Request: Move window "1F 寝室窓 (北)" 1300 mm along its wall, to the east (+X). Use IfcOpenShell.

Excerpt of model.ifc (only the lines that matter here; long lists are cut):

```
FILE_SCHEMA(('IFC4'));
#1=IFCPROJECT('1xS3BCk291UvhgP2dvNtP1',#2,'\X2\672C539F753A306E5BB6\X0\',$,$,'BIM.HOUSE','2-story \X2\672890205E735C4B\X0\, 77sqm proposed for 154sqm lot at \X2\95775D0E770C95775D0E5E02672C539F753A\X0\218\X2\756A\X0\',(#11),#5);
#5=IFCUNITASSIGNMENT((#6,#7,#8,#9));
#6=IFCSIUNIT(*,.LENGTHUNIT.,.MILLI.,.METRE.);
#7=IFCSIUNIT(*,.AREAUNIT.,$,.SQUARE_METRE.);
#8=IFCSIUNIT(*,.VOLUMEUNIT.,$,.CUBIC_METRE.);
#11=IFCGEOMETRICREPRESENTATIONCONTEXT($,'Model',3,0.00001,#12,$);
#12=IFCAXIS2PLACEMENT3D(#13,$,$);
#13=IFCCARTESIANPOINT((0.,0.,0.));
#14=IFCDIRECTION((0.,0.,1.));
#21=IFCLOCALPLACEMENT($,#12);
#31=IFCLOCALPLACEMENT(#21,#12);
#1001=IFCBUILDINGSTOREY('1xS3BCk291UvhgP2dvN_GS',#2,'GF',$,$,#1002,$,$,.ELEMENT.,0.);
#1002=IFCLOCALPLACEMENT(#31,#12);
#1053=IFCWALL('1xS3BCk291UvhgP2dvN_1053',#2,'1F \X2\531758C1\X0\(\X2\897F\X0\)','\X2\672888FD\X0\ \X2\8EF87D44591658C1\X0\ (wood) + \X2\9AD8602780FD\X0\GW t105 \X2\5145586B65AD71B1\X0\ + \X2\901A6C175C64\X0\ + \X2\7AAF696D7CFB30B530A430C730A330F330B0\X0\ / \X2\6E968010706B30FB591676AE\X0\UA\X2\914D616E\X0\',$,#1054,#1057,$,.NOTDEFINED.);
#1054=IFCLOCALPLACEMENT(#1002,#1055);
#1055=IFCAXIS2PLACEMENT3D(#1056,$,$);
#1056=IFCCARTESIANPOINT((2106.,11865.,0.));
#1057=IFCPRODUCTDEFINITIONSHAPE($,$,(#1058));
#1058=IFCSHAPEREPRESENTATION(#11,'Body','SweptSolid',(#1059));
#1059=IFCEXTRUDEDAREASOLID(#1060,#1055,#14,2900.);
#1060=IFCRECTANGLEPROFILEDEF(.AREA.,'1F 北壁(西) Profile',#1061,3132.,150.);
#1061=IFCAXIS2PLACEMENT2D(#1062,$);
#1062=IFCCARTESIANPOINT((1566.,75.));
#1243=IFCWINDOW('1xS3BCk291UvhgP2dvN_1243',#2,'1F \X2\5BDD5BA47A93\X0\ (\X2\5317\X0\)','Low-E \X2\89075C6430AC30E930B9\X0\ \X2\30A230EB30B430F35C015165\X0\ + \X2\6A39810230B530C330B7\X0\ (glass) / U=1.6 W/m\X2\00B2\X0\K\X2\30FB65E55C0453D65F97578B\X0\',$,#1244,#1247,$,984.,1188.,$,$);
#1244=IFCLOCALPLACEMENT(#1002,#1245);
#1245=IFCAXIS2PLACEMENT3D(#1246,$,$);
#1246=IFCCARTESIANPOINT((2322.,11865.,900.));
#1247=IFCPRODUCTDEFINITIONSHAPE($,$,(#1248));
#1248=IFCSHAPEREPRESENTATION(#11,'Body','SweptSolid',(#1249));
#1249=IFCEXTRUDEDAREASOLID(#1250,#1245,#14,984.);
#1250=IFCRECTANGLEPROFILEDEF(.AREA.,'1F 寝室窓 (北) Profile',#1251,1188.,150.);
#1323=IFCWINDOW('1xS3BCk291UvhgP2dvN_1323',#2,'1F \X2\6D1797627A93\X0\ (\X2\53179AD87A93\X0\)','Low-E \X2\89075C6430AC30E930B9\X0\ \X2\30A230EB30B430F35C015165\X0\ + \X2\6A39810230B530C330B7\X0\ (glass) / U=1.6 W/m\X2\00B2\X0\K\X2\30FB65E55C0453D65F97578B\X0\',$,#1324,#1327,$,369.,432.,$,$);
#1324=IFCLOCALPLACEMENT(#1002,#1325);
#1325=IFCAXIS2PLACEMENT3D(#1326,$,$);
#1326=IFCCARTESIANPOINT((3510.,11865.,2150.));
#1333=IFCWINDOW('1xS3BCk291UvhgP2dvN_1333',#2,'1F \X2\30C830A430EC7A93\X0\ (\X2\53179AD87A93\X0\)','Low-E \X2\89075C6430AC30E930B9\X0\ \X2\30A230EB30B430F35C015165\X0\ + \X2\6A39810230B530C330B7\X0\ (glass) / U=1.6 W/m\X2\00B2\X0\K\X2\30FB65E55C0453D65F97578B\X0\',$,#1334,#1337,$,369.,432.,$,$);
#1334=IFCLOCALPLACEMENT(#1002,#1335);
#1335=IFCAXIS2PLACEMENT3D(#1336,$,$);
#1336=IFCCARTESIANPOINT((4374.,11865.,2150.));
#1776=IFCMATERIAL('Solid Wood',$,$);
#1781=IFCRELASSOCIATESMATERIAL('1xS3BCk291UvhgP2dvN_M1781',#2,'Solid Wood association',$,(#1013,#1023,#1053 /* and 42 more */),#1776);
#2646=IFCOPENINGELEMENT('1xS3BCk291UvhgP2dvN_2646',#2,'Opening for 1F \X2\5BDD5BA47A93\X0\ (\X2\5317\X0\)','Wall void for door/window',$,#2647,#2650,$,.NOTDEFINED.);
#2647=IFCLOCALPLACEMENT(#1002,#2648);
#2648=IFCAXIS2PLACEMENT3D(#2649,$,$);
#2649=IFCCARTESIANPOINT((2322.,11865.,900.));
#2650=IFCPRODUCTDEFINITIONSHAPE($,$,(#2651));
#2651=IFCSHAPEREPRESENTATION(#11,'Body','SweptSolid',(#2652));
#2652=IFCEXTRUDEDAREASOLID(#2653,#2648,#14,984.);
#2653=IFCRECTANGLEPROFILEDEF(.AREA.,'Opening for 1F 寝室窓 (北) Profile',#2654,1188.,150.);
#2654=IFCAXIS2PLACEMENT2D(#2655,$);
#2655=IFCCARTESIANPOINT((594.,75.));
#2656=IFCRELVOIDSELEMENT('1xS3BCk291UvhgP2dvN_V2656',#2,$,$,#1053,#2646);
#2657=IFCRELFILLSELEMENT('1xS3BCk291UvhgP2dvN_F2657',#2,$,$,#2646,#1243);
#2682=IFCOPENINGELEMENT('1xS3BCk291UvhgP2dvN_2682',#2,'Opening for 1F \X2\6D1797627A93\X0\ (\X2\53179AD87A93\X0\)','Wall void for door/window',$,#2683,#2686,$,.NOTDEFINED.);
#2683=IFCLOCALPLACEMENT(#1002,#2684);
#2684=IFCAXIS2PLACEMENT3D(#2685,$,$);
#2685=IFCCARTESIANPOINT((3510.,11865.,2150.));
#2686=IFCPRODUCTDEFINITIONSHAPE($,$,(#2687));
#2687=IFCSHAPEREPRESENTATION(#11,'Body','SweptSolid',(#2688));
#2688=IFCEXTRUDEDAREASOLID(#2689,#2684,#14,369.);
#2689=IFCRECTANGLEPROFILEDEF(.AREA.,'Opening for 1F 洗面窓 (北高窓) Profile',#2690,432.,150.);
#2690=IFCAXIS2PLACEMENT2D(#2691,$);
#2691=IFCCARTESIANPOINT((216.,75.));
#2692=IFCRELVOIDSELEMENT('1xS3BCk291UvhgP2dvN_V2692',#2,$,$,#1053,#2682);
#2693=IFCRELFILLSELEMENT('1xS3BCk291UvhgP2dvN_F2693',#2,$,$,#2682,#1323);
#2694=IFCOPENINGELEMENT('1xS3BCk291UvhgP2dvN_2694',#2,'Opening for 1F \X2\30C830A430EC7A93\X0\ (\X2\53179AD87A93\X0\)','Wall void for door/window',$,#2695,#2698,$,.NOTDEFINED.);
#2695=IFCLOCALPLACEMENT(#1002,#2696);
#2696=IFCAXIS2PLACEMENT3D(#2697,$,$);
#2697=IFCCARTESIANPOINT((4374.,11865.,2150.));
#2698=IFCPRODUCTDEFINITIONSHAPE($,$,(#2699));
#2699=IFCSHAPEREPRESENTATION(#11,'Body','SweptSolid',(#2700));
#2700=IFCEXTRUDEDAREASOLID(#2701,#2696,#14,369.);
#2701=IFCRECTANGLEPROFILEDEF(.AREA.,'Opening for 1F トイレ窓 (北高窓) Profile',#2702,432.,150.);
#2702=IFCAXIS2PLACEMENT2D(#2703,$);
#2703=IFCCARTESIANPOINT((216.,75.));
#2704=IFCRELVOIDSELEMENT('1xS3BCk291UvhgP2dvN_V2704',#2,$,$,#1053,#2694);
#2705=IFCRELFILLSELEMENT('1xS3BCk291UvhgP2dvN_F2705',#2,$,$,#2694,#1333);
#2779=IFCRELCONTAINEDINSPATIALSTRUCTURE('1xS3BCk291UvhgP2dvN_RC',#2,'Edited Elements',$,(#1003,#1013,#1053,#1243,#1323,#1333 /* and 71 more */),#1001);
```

```python
import ifcopenshell
import ifcopenshell.api.geometry
import ifcopenshell.util.placement

model = ifcopenshell.open("model.ifc")

window = model.by_guid("1xS3BCk291UvhgP2dvN_1243")
opening = window.FillsVoids[0].RelatingOpeningElement
wall = opening.VoidsElements[0].RelatingBuildingElement

wall_matrix = ifcopenshell.util.placement.get_local_placement(wall.ObjectPlacement)
shift = wall_matrix[:3, 0] * 1300.0
before = ifcopenshell.util.placement.get_local_placement(window.ObjectPlacement)[:3, 3].copy()

# The window is not placed relative to its opening, so move both.
for product in (opening, window):
    matrix = ifcopenshell.util.placement.get_local_placement(product.ObjectPlacement)
    matrix[:3, 3] += shift
    ifcopenshell.api.geometry.edit_object_placement(model, product=product, matrix=matrix, is_si=False)

after = ifcopenshell.util.placement.get_local_placement(window.ObjectPlacement)[:3, 3]
print("window moved by", (after - before).round(3) + 0.0)

model.write("model_updated.ifc")
```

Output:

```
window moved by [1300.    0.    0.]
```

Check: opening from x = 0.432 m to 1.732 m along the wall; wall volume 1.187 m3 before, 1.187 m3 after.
